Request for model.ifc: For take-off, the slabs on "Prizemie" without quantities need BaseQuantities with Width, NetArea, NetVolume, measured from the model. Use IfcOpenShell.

First a look at what the model holds.

```python
import ifcopenshell
import ifcopenshell.util.element
import ifcopenshell.util.unit

model = ifcopenshell.open("model.ifc")
print(model.schema)
for unit_type in ("LENGTHUNIT", "AREAUNIT", "VOLUMEUNIT"):
    print(unit_type, ifcopenshell.util.unit.calculate_unit_scale(model, unit_type))
storey = next(s for s in model.by_type("IfcBuildingStorey") if s.Name == "Prizemie")
slabs = [e for e in ifcopenshell.util.element.get_decomposition(storey) if e.is_a("IfcSlab")]
for e in sorted(slabs, key=lambda e: e.id()):
    print(e.id(), e.is_a(), e.Name, list(ifcopenshell.util.element.get_psets(e, qtos_only=True)), sep=" | ")
```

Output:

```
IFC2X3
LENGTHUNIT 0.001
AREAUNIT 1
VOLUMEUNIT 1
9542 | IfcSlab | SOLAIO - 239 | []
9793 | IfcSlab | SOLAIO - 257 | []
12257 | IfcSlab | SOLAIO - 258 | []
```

```python
import ifcopenshell
import ifcopenshell.api.pset
import ifcopenshell.geom
import ifcopenshell.util.element
import ifcopenshell.util.shape
import ifcopenshell.util.unit

model = ifcopenshell.open("model.ifc")
unit_scale = ifcopenshell.util.unit.calculate_unit_scale(model)
area_scale = ifcopenshell.util.unit.calculate_unit_scale(model, "AREAUNIT")
volume_scale = ifcopenshell.util.unit.calculate_unit_scale(model, "VOLUMEUNIT")
settings = ifcopenshell.geom.settings()

storey = next(s for s in model.by_type("IfcBuildingStorey") if s.Name == "Prizemie")
slabs = [e for e in ifcopenshell.util.element.get_decomposition(storey) if e.is_a("IfcSlab")]

for e in sorted(slabs, key=lambda e: e.id()):
    if ifcopenshell.util.element.get_psets(e, qtos_only=True, should_inherit=False):
        continue
    # Geometry comes back in metres, in the element's own axes.
    shape = ifcopenshell.geom.create_shape(settings, e)
    values = {
        "Width": ifcopenshell.util.shape.get_z(shape.geometry) / unit_scale,
        "NetArea": ifcopenshell.util.shape.get_footprint_area(shape.geometry) / area_scale,
        "NetVolume": ifcopenshell.util.shape.get_volume(shape.geometry) / volume_scale,
    }
    qto = ifcopenshell.api.pset.add_qto(model, product=e, name="BaseQuantities")
    ifcopenshell.api.pset.edit_qto(model, qto=qto, properties=values)
    print(e.id(), {k: round(v, 3) for k, v in values.items()})

model.write("model_v2.ifc")
```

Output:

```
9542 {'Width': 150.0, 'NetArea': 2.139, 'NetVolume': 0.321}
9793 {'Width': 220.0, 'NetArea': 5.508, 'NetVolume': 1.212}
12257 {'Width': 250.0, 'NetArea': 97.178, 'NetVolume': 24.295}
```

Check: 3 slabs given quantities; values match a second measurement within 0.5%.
